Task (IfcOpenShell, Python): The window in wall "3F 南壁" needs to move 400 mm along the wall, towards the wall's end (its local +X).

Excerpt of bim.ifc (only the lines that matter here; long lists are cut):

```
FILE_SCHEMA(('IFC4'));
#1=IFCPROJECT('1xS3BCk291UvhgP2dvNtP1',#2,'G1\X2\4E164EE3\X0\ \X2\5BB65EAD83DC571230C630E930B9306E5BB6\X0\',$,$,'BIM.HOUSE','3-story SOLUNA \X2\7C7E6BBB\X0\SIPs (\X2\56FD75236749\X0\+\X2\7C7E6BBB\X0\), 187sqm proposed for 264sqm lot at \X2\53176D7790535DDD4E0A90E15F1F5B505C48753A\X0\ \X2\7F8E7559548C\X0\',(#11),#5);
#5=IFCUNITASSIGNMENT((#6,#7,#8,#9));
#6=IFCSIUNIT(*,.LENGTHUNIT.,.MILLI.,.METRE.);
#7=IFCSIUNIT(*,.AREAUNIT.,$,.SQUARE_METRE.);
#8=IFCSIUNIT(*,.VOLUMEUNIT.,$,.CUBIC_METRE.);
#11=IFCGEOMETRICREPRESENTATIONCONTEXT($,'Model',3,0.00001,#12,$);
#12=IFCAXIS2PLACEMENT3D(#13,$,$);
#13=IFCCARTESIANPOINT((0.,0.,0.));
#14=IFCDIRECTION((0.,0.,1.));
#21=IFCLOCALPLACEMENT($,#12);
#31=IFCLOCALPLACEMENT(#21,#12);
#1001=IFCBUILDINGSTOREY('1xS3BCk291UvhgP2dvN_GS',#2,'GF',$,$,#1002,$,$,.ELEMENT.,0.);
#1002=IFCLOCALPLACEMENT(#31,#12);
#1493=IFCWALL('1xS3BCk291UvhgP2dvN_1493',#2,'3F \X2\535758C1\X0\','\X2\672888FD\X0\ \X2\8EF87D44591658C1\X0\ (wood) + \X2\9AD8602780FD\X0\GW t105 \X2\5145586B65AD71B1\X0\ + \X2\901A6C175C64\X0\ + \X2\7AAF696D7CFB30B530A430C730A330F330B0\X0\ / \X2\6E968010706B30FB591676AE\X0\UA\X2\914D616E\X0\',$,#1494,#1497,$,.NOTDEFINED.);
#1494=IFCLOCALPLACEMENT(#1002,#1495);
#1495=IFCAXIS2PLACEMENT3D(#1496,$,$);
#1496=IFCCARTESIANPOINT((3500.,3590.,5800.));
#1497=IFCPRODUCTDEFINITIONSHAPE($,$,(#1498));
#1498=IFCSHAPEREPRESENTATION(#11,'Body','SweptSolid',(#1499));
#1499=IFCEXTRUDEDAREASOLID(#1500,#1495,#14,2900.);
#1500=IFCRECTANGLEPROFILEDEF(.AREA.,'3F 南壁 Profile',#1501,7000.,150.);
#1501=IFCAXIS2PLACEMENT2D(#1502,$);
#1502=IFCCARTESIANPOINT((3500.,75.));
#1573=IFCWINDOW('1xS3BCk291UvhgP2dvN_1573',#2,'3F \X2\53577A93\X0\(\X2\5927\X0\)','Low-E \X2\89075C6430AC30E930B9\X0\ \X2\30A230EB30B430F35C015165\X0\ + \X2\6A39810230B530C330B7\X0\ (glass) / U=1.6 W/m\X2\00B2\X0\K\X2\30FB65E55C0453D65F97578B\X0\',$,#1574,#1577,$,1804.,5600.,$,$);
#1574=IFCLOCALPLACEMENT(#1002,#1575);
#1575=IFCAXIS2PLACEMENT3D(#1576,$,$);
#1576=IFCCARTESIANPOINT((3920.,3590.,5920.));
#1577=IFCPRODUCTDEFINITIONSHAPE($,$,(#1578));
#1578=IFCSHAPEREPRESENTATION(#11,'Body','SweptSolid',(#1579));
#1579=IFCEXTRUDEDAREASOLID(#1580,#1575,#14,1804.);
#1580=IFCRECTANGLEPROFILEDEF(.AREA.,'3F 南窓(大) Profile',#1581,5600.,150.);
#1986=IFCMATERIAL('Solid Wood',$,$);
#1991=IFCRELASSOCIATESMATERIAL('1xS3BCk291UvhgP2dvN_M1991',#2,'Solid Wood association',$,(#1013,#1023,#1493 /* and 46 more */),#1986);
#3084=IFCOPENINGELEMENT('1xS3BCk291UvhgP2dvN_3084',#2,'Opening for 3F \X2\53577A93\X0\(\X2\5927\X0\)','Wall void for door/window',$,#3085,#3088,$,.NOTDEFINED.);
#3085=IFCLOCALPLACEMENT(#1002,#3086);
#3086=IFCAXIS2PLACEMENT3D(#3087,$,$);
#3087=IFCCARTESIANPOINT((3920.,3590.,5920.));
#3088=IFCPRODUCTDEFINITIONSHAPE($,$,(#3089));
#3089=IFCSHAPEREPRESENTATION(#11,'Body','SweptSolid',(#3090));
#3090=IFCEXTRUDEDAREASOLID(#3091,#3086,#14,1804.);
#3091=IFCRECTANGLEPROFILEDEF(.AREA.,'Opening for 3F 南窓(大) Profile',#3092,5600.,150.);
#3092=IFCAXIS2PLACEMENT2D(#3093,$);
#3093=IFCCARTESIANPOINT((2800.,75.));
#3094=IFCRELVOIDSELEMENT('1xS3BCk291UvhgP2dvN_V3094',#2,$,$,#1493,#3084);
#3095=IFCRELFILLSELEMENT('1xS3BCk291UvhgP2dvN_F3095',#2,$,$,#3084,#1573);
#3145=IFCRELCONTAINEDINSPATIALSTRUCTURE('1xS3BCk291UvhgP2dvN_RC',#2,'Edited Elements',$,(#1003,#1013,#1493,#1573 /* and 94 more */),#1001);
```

```python
import ifcopenshell
import ifcopenshell.api.geometry
import ifcopenshell.util.placement
import ifcopenshell.util.unit

model = ifcopenshell.open("bim.ifc")
unit_scale = ifcopenshell.util.unit.calculate_unit_scale(model)

window = model.by_guid("1xS3BCk291UvhgP2dvN_1573")
opening = window.FillsVoids[0].RelatingOpeningElement
wall = opening.VoidsElements[0].RelatingBuildingElement

wall_matrix = ifcopenshell.util.placement.get_local_placement(wall.ObjectPlacement)
shift = wall_matrix[:3, 0] * 0.4 / unit_scale
before = ifcopenshell.util.placement.get_local_placement(window.ObjectPlacement)[:3, 3].copy()

# The window is not placed relative to its opening, so move both.
for product in (opening, window):
    matrix = ifcopenshell.util.placement.get_local_placement(product.ObjectPlacement)
    matrix[:3, 3] += shift
    ifcopenshell.api.geometry.edit_object_placement(model, product=product, matrix=matrix, is_si=False)

after = ifcopenshell.util.placement.get_local_placement(window.ObjectPlacement)[:3, 3]
print("window moved by", (after - before).round(3) + 0.0)

model.write("bim_v2.ifc")
```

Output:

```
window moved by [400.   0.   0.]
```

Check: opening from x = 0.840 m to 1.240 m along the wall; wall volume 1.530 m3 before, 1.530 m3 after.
